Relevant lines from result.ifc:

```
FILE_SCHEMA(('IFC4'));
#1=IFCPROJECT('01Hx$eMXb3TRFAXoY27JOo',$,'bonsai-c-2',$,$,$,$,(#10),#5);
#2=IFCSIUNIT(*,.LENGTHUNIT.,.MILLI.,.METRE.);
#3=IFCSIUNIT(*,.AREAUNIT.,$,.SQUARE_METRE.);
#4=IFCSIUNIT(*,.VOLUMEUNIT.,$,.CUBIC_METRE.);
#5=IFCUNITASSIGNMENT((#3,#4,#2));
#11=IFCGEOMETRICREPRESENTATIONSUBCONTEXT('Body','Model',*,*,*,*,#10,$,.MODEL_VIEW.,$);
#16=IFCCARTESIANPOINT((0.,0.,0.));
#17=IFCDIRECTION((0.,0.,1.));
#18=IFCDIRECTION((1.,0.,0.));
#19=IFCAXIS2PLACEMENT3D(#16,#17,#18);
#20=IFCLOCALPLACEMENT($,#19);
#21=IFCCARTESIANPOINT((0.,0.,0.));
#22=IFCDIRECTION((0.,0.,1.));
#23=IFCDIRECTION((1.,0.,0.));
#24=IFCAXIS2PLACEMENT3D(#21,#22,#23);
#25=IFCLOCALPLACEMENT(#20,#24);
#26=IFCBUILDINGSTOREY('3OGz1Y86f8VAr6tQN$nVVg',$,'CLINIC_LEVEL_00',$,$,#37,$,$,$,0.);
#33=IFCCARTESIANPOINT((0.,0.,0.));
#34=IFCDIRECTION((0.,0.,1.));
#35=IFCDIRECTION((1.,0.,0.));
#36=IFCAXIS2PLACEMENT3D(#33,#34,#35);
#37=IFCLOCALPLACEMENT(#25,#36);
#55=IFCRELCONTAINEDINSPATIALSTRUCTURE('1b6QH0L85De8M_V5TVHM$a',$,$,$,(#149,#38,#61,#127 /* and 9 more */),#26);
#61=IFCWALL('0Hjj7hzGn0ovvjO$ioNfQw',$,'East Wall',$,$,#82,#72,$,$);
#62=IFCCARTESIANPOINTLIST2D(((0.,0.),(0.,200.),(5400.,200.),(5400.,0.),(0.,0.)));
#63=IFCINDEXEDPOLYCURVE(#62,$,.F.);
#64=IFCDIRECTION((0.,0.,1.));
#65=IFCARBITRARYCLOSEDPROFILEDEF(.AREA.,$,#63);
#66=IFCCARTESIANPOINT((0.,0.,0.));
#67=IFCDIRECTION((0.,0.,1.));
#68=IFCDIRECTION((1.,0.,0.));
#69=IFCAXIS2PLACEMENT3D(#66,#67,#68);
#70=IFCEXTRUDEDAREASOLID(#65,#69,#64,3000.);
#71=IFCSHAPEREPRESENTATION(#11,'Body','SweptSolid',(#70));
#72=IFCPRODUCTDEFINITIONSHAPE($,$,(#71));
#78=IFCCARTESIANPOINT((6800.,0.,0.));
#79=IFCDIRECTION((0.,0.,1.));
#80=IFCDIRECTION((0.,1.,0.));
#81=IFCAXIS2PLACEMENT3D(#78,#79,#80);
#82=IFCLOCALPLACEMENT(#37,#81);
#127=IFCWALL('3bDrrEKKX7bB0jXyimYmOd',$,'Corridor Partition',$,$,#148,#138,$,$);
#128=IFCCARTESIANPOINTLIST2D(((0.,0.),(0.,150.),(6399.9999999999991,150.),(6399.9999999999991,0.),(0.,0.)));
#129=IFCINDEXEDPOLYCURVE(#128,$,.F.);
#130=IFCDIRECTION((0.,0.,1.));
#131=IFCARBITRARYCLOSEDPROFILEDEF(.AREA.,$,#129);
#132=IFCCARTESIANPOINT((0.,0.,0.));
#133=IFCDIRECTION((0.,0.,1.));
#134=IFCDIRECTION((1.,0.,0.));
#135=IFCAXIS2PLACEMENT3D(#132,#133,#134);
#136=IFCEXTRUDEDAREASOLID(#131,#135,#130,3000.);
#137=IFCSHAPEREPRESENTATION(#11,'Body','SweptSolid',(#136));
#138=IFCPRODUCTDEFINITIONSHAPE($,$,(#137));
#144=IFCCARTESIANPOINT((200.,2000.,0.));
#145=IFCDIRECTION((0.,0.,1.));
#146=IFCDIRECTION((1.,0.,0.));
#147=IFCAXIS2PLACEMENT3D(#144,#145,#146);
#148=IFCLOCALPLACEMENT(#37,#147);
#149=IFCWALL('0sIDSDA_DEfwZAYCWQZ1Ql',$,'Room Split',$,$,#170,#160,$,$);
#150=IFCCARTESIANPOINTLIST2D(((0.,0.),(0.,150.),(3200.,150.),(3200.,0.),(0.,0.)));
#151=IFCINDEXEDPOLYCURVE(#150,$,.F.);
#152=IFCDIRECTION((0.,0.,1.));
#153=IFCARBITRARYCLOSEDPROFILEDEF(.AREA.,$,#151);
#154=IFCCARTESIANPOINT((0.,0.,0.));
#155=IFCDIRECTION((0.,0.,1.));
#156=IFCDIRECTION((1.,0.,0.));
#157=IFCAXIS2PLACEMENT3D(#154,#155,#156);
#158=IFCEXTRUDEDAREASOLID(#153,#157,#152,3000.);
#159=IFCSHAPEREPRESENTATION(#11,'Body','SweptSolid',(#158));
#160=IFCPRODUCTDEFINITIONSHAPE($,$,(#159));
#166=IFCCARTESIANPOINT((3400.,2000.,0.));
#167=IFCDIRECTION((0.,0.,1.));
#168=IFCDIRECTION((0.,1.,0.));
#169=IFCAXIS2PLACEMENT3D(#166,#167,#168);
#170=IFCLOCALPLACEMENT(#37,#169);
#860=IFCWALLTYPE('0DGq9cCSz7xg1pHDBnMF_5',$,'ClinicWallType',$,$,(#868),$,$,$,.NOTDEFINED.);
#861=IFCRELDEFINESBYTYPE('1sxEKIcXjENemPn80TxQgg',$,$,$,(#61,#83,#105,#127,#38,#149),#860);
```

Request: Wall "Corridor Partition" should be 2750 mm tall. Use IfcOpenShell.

```python
import ifcopenshell
import ifcopenshell.geom
import ifcopenshell.util.representation
import ifcopenshell.util.shape

model = ifcopenshell.open("result.ifc")
settings = ifcopenshell.geom.settings()


def volume(element):
    """Net volume in cubic metres, openings subtracted."""
    shape = ifcopenshell.geom.create_shape(settings, element)
    return ifcopenshell.util.shape.get_volume(shape.geometry)


wall = model.by_id(127)
before = volume(wall)

body = ifcopenshell.util.representation.get_representation(wall, "Model", "Body")
solid = body.Items[0]
old_height = solid.Depth
solid.Depth = 2750.0
after = volume(wall)

print(f"height {old_height:g} -> {solid.Depth:g}, volume {before:.3f} -> {after:.3f} m3")

model.write("result_rev.ifc")
```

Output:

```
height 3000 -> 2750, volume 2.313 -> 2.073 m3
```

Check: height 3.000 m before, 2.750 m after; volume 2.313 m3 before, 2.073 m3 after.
